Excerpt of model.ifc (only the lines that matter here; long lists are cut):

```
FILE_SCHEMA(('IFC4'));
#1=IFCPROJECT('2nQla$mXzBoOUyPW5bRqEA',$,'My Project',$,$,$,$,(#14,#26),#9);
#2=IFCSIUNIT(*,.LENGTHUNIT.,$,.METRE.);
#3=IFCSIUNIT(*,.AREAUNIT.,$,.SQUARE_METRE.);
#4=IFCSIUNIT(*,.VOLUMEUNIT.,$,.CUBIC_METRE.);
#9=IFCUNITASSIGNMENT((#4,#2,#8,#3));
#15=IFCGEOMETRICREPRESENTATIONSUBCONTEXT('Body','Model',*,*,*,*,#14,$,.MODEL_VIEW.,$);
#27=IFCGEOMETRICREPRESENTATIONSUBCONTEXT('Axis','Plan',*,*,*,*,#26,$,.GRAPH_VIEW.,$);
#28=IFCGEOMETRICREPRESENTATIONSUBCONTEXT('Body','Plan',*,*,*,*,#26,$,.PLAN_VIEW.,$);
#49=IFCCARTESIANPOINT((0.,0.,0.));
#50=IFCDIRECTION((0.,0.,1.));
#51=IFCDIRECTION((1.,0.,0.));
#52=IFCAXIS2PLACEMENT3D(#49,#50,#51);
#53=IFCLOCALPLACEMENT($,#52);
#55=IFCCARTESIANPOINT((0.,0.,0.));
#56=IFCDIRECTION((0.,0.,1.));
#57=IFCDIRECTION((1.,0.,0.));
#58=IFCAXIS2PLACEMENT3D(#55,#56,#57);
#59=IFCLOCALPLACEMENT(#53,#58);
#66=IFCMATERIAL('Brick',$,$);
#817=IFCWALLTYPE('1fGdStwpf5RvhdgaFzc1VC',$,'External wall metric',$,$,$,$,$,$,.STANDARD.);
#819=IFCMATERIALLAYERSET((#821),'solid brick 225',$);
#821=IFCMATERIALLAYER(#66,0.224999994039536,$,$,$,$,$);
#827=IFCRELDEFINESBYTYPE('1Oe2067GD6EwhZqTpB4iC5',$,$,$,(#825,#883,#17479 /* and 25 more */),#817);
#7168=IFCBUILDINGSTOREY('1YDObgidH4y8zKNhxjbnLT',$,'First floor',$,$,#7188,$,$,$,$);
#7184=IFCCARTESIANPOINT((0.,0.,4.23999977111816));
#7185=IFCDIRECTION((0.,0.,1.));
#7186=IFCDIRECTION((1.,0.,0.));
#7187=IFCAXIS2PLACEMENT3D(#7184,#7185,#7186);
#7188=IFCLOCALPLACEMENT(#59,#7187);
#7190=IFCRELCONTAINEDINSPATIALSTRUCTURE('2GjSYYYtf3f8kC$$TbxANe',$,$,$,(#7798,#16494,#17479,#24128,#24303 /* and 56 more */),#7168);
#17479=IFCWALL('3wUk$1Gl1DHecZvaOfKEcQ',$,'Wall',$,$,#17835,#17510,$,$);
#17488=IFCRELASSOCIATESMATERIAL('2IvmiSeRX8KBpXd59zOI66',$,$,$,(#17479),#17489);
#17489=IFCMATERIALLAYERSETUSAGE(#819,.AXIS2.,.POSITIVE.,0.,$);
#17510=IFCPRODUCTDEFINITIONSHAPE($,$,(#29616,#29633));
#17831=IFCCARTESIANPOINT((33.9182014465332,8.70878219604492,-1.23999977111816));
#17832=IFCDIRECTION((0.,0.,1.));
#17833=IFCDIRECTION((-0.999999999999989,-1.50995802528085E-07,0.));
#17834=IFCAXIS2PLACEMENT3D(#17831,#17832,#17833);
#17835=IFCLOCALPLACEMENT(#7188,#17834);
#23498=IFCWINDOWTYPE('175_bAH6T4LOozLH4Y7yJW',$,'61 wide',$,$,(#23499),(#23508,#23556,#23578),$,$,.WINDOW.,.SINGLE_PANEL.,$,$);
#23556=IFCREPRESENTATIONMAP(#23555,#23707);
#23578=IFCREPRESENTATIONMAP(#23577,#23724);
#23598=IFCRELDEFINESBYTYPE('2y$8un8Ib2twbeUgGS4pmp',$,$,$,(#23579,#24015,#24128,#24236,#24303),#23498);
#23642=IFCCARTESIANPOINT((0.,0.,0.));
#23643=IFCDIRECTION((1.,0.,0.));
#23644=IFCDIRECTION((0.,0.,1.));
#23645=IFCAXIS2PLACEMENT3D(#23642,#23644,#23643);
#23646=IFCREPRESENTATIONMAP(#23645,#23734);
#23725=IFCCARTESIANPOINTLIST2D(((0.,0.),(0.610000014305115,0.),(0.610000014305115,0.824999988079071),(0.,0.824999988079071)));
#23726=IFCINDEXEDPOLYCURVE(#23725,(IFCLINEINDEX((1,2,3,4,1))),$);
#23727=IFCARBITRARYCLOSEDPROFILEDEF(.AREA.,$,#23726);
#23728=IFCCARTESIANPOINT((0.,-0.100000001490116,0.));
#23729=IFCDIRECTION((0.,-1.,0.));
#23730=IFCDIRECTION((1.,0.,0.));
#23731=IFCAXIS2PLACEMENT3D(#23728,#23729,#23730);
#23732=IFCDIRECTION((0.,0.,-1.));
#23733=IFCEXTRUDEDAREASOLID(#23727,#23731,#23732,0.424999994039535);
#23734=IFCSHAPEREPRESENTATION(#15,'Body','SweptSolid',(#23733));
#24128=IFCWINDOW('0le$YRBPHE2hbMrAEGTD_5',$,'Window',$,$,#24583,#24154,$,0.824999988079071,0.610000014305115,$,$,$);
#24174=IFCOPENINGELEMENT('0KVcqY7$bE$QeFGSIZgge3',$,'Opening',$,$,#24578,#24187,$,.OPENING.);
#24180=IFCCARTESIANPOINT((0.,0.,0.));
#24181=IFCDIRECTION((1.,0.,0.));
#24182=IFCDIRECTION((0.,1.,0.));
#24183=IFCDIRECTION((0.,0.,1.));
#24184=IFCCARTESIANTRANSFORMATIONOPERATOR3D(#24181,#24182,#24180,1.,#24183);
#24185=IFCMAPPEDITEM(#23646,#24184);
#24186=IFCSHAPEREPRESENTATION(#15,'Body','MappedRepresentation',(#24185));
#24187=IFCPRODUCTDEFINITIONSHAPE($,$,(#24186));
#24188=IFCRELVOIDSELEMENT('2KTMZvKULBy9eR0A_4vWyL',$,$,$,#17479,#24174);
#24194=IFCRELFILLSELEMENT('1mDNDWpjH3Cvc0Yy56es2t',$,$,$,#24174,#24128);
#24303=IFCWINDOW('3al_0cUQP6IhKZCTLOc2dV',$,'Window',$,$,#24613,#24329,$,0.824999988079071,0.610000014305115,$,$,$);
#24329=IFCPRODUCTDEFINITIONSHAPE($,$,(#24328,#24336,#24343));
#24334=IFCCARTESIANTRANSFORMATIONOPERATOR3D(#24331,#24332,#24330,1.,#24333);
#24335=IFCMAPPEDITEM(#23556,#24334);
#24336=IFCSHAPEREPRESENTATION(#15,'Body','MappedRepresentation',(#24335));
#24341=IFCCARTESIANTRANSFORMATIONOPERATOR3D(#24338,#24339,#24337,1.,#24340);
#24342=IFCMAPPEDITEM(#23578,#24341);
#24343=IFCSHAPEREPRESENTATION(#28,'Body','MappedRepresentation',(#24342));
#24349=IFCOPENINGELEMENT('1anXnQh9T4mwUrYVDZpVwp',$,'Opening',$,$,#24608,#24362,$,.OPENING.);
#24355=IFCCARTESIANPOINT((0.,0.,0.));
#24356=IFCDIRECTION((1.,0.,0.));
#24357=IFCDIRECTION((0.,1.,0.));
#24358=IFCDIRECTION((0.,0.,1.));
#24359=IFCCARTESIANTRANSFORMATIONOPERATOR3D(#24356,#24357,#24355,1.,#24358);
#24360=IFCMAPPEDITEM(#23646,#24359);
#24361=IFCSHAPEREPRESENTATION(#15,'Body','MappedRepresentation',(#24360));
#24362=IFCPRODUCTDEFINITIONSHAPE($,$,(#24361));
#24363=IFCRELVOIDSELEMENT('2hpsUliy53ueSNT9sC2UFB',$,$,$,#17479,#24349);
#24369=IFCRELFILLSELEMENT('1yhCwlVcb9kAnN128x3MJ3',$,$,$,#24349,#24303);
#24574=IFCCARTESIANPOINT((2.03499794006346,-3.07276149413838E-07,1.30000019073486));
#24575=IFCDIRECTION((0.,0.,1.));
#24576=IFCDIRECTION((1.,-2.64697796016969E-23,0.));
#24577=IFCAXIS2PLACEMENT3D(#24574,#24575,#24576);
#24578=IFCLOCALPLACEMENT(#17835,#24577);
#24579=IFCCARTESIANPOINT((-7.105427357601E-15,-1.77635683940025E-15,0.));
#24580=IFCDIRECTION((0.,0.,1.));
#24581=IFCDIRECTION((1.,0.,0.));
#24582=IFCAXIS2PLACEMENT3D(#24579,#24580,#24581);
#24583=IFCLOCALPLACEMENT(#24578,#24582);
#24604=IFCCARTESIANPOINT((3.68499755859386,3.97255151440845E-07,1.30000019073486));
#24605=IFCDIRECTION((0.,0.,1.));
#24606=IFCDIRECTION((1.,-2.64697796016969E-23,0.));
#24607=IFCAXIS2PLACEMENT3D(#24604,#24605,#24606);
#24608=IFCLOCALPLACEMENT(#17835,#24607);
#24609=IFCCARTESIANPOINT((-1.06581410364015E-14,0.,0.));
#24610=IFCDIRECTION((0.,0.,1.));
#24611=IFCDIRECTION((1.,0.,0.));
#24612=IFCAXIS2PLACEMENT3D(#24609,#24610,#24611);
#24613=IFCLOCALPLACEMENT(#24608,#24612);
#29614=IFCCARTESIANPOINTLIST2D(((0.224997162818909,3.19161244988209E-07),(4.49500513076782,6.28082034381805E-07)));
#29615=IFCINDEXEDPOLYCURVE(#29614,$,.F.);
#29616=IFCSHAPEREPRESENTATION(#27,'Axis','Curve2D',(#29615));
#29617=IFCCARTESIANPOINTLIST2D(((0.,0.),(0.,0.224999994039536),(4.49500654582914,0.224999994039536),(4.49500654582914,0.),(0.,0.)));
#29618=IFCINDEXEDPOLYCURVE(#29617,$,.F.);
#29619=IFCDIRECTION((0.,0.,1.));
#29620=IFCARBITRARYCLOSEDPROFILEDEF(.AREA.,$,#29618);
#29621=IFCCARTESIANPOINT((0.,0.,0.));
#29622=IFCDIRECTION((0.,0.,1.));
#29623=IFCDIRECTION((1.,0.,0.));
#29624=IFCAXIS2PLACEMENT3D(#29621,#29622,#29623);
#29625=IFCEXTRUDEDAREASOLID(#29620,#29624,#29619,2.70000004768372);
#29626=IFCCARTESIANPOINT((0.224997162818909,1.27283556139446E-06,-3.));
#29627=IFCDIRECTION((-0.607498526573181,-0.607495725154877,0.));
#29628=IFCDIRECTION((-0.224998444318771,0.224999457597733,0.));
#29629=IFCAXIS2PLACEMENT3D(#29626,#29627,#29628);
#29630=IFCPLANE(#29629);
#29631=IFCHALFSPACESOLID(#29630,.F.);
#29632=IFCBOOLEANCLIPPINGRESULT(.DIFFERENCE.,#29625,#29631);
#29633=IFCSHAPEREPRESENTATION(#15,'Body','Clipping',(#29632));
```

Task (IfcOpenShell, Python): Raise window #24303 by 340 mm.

```python
import numpy as np
import ifcopenshell
import ifcopenshell.api.geometry
import ifcopenshell.util.placement
import ifcopenshell.util.unit

model = ifcopenshell.open("model.ifc")
unit_scale = ifcopenshell.util.unit.calculate_unit_scale(model)

window = model.by_guid("3al_0cUQP6IhKZCTLOc2dV")
opening = window.FillsVoids[0].RelatingOpeningElement
dz = 0.34 / unit_scale

shift = np.array([0.0, 0.0, dz])
# The window is placed relative to its opening, so it follows when the opening moves.
matrix = ifcopenshell.util.placement.get_local_placement(opening.ObjectPlacement)
matrix[:3, 3] += shift
ifcopenshell.api.geometry.edit_object_placement(
    model, product=opening, matrix=matrix, is_si=False, should_transform_children=True
)

print(f"moved by {dz * unit_scale:+.3f} m")

model.write("model-out.ifc")
```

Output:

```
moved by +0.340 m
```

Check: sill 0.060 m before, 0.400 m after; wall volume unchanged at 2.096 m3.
